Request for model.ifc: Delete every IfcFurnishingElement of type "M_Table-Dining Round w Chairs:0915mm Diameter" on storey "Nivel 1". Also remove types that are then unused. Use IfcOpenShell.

First a look at what the model holds.

```python
import ifcopenshell
import ifcopenshell.util.element

model = ifcopenshell.open("model.ifc")
print(model.schema)
storey = next(s for s in model.by_type("IfcBuildingStorey") if s.Name == "Nivel 1")
furniture = [e for e in ifcopenshell.util.element.get_decomposition(storey) if e.is_a("IfcFurnishingElement")]
seen = {}
for e in furniture:
    element_type = ifcopenshell.util.element.get_type(e)
    name = element_type.Name if element_type not in (None, e) else None
    seen[name] = seen.get(name, 0) + 1
for name, count in sorted(seen.items(), key=str):
    print(count, "x", name)
```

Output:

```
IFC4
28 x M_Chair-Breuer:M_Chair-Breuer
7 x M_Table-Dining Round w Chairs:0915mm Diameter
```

```python
import ifcopenshell
import ifcopenshell.api.root
import ifcopenshell.util.element

model = ifcopenshell.open("model.ifc")

storey = next(s for s in model.by_type("IfcBuildingStorey") if s.Name == "Nivel 1")
furniture = [e for e in ifcopenshell.util.element.get_decomposition(storey) if e.is_a("IfcFurnishingElement")]
targets = [e for e in furniture if (t := ifcopenshell.util.element.get_type(e)) not in (None, e) and t.Name == "M_Table-Dining Round w Chairs:0915mm Diameter"]
types = {ifcopenshell.util.element.get_type(e) for e in targets} - {None, *targets}

for e in targets:
    ifcopenshell.api.root.remove_product(model, product=e)
print(len(targets), "removed")

unused = [t for t in types if not ifcopenshell.util.element.get_types(t)]
for t in unused:
    ifcopenshell.api.root.remove_product(model, product=t)
print(len(unused), "unused types removed")

model.write("model_v2.ifc")
```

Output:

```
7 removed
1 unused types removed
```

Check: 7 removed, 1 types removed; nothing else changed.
